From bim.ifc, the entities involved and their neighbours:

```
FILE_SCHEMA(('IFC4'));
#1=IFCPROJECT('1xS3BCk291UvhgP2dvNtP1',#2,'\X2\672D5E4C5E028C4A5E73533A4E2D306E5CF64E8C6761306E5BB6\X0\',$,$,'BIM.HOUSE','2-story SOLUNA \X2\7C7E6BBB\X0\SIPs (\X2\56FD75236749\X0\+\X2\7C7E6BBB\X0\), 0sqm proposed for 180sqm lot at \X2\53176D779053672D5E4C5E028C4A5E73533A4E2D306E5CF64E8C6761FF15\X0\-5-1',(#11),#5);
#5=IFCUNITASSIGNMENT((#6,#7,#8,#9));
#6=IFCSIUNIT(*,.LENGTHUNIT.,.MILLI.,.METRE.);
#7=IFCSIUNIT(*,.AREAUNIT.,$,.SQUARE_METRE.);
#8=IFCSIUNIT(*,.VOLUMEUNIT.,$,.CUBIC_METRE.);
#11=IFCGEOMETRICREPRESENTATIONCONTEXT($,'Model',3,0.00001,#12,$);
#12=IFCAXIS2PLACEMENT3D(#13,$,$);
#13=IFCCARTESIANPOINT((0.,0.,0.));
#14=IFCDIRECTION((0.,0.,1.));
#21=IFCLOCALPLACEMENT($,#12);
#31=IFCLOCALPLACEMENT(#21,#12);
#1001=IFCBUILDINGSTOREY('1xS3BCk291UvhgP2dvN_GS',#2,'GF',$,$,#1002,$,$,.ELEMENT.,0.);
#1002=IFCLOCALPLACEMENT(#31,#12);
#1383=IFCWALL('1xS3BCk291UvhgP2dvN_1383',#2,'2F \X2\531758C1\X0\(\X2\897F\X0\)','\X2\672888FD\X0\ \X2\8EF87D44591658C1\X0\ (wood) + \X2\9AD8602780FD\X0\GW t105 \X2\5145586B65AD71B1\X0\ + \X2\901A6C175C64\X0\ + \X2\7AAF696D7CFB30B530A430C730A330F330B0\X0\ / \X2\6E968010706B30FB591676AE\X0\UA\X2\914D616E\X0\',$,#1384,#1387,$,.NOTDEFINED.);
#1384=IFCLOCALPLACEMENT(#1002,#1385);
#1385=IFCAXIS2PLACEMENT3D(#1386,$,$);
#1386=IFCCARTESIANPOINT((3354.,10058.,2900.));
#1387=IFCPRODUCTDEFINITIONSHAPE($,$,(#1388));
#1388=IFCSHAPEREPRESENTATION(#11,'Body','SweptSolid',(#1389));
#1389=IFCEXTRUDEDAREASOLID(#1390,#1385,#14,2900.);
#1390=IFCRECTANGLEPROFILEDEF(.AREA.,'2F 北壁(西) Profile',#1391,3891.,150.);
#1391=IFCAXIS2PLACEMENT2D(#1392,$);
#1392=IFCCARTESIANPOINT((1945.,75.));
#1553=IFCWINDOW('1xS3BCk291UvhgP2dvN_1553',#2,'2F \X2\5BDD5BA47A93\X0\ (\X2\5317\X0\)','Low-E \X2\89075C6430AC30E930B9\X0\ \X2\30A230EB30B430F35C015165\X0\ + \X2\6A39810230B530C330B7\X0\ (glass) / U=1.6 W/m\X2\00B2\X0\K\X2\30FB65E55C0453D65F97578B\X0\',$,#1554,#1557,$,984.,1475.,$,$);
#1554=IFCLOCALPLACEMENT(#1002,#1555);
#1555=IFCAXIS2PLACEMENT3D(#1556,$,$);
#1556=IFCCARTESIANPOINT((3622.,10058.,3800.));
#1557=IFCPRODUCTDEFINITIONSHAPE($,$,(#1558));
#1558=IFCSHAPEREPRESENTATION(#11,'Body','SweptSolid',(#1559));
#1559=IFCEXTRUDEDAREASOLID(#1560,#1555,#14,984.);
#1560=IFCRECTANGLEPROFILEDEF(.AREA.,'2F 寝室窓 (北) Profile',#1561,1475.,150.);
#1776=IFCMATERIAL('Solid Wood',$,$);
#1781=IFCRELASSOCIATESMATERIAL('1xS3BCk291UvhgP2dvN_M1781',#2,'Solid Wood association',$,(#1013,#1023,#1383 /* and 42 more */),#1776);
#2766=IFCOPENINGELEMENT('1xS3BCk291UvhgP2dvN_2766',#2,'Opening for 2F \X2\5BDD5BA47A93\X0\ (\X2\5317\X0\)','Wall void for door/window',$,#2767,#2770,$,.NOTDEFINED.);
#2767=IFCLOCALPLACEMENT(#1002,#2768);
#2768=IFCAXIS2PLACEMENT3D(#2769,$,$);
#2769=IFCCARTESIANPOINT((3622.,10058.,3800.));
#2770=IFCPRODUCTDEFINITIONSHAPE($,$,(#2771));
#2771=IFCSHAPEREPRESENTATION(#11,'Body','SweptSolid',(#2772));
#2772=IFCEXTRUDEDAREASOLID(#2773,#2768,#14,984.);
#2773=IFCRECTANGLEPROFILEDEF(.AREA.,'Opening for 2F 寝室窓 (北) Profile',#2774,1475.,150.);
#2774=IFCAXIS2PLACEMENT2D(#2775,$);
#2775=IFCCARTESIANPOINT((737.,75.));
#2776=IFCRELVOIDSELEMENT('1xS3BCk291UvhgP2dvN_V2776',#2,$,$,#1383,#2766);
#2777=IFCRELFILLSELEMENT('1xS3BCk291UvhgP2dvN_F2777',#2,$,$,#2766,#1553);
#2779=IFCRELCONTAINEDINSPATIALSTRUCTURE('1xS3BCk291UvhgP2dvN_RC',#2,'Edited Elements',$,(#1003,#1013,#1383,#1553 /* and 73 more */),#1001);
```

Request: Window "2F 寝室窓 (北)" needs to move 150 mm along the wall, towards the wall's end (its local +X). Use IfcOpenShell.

```python
import ifcopenshell
import ifcopenshell.api.geometry
import ifcopenshell.util.placement
import ifcopenshell.util.unit

model = ifcopenshell.open("bim.ifc")
unit_scale = ifcopenshell.util.unit.calculate_unit_scale(model)

window = model.by_guid("1xS3BCk291UvhgP2dvN_1553")
opening = window.FillsVoids[0].RelatingOpeningElement
wall = opening.VoidsElements[0].RelatingBuildingElement

wall_matrix = ifcopenshell.util.placement.get_local_placement(wall.ObjectPlacement)
shift = wall_matrix[:3, 0] * 0.15 / unit_scale
before = ifcopenshell.util.placement.get_local_placement(window.ObjectPlacement)[:3, 3].copy()

# The window is not placed relative to its opening, so move both.
for product in (opening, window):
    matrix = ifcopenshell.util.placement.get_local_placement(product.ObjectPlacement)
    matrix[:3, 3] += shift
    ifcopenshell.api.geometry.edit_object_placement(model, product=product, matrix=matrix, is_si=False)

after = ifcopenshell.util.placement.get_local_placement(window.ObjectPlacement)[:3, 3]
print("window moved by", (after - before).round(3) + 0.0)

model.write("bim-out.ifc")
```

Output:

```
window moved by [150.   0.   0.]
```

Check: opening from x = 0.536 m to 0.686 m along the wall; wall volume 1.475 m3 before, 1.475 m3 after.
